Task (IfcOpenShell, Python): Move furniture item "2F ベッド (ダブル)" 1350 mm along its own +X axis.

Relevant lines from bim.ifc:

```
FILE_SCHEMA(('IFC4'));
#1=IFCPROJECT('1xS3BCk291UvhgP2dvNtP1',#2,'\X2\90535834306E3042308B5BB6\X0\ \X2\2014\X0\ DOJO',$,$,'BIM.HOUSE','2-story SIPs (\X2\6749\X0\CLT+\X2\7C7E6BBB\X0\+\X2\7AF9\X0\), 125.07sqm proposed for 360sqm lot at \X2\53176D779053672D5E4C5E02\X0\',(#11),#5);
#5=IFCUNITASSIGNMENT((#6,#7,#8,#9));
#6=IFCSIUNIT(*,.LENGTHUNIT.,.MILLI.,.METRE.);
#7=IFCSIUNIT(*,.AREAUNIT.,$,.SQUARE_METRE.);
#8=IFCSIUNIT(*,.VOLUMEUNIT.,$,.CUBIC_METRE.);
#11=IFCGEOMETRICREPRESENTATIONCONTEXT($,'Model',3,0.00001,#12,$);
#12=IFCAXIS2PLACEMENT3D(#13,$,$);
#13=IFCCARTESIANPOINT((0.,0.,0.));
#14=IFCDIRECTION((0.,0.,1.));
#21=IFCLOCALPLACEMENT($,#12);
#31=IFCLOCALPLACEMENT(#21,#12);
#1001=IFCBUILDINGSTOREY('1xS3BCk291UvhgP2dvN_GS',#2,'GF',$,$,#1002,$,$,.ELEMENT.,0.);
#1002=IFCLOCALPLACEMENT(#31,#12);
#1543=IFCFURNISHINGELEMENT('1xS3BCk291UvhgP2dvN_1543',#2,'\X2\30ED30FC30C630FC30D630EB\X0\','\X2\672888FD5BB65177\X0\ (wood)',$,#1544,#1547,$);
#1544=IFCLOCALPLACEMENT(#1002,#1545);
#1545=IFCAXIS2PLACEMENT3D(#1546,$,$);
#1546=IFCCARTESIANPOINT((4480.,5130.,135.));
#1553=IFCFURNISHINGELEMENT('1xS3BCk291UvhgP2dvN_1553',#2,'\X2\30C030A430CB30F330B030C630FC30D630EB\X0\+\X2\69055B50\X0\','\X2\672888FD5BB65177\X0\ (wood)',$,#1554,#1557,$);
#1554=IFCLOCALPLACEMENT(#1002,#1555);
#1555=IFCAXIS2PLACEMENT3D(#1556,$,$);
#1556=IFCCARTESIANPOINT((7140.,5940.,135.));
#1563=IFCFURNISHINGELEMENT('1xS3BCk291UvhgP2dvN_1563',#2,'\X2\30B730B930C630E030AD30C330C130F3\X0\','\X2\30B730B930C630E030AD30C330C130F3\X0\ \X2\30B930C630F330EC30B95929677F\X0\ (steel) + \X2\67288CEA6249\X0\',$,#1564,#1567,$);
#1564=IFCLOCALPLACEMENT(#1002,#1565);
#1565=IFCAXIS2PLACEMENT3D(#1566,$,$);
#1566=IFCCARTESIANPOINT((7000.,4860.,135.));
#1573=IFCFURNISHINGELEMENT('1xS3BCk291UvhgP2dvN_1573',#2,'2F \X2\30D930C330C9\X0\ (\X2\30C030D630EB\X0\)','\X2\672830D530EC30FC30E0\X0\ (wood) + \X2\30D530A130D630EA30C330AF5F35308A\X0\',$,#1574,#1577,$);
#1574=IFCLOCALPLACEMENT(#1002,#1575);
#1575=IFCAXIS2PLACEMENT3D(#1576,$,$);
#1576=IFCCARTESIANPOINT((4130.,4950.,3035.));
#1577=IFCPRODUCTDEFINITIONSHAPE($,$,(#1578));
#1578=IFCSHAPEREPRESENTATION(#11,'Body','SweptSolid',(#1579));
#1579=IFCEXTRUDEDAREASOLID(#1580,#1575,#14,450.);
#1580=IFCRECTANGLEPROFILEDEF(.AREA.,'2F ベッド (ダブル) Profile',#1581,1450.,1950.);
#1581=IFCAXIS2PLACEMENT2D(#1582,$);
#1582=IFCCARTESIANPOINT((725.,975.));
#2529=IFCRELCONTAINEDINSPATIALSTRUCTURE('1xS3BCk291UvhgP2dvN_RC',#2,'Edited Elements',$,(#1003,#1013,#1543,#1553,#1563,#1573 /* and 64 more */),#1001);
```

```python
import ifcopenshell
import ifcopenshell.api.geometry
import ifcopenshell.util.placement

model = ifcopenshell.open("bim.ifc")

item = model.by_guid("1xS3BCk291UvhgP2dvN_1573")
matrix = ifcopenshell.util.placement.get_local_placement(item.ObjectPlacement)
matrix[:3, 3] += matrix[:3, 0] * 1350.0
ifcopenshell.api.geometry.edit_object_placement(model, product=item, matrix=matrix, is_si=False)

print(ifcopenshell.util.placement.get_local_placement(item.ObjectPlacement).round(3) + 0.0)

model.write("bim_updated.ifc")
```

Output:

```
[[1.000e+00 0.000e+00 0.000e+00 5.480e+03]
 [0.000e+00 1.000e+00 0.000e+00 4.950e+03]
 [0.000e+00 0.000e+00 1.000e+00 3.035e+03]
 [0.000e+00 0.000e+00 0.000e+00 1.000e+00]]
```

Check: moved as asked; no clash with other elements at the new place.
